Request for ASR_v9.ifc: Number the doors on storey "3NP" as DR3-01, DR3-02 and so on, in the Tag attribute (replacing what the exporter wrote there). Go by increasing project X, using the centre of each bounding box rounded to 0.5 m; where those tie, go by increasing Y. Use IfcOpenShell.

First a look at what the model holds.

```python
import ifcopenshell
import ifcopenshell.util.element
import ifcopenshell.util.placement

model = ifcopenshell.open("ASR_v9.ifc")
print(model.schema)
storey = next(s for s in model.by_type("IfcBuildingStorey") if s.Name == "3NP")
doors = [e for e in ifcopenshell.util.element.get_decomposition(storey) if e.is_a("IfcDoor")]
for e in sorted(doors, key=lambda e: e.id()):
    origin = ifcopenshell.util.placement.get_local_placement(e.ObjectPlacement)[:3, 3]
    print(e.id(), e.Tag, e.Name, origin.round(2) + 0.0, sep=" | ")
```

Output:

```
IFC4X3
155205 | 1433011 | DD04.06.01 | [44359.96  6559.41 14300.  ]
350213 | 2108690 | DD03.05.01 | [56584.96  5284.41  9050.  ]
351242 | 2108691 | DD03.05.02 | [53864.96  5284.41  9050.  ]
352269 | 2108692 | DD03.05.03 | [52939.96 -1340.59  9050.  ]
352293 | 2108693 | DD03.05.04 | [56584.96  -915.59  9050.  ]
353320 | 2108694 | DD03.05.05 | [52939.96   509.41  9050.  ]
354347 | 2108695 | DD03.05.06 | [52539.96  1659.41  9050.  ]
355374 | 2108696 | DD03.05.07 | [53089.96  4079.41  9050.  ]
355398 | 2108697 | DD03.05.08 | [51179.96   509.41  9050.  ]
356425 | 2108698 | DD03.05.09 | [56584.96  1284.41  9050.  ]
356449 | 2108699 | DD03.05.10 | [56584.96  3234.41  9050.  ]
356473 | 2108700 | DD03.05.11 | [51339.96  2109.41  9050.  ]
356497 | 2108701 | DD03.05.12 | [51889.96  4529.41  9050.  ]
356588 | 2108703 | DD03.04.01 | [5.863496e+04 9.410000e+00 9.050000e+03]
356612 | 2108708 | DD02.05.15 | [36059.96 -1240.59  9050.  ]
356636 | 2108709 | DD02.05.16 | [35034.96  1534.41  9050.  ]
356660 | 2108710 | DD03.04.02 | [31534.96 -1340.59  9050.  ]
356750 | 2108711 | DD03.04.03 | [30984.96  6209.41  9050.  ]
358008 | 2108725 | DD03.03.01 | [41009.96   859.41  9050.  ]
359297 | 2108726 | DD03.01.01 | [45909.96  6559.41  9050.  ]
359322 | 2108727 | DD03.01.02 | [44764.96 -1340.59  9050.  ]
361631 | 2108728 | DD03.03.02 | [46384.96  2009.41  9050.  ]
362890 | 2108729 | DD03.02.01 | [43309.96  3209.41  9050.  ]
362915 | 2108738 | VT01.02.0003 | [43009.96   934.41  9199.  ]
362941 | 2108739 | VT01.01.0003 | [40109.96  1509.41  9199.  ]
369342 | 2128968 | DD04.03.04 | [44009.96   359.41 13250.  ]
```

```python
import ifcopenshell
import ifcopenshell.geom
import ifcopenshell.util.element
import ifcopenshell.util.shape

model = ifcopenshell.open("ASR_v9.ifc")
settings = ifcopenshell.geom.settings()
settings.set("use-world-coords", True)


def centre(element):
    shape = ifcopenshell.geom.create_shape(settings, element)
    return ifcopenshell.util.shape.get_bbox_centroid(shape.geometry)


storey = next(s for s in model.by_type("IfcBuildingStorey") if s.Name == "3NP")
doors = [e for e in ifcopenshell.util.element.get_decomposition(storey) if e.is_a("IfcDoor")]

# Insertion points can sit at a corner or the storey origin, so sort by the geometry (in metres).
centres = {e: centre(e) for e in doors}
doors.sort(key=lambda e: (round(centres[e][0] / 0.5), centres[e][1]))

for i, e in enumerate(doors, start=1):
    number = f"DR3-{i:02d}"
    e.Tag = number
    print(e.id(), number)

model.write("ASR_v9-out.ifc")
```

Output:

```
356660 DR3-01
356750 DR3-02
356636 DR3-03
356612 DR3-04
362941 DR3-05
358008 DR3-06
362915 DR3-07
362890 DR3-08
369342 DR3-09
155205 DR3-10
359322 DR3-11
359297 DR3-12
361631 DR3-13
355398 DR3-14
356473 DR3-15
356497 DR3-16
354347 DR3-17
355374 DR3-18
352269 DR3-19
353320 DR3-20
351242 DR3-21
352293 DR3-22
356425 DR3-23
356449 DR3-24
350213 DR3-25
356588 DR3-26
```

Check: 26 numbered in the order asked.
